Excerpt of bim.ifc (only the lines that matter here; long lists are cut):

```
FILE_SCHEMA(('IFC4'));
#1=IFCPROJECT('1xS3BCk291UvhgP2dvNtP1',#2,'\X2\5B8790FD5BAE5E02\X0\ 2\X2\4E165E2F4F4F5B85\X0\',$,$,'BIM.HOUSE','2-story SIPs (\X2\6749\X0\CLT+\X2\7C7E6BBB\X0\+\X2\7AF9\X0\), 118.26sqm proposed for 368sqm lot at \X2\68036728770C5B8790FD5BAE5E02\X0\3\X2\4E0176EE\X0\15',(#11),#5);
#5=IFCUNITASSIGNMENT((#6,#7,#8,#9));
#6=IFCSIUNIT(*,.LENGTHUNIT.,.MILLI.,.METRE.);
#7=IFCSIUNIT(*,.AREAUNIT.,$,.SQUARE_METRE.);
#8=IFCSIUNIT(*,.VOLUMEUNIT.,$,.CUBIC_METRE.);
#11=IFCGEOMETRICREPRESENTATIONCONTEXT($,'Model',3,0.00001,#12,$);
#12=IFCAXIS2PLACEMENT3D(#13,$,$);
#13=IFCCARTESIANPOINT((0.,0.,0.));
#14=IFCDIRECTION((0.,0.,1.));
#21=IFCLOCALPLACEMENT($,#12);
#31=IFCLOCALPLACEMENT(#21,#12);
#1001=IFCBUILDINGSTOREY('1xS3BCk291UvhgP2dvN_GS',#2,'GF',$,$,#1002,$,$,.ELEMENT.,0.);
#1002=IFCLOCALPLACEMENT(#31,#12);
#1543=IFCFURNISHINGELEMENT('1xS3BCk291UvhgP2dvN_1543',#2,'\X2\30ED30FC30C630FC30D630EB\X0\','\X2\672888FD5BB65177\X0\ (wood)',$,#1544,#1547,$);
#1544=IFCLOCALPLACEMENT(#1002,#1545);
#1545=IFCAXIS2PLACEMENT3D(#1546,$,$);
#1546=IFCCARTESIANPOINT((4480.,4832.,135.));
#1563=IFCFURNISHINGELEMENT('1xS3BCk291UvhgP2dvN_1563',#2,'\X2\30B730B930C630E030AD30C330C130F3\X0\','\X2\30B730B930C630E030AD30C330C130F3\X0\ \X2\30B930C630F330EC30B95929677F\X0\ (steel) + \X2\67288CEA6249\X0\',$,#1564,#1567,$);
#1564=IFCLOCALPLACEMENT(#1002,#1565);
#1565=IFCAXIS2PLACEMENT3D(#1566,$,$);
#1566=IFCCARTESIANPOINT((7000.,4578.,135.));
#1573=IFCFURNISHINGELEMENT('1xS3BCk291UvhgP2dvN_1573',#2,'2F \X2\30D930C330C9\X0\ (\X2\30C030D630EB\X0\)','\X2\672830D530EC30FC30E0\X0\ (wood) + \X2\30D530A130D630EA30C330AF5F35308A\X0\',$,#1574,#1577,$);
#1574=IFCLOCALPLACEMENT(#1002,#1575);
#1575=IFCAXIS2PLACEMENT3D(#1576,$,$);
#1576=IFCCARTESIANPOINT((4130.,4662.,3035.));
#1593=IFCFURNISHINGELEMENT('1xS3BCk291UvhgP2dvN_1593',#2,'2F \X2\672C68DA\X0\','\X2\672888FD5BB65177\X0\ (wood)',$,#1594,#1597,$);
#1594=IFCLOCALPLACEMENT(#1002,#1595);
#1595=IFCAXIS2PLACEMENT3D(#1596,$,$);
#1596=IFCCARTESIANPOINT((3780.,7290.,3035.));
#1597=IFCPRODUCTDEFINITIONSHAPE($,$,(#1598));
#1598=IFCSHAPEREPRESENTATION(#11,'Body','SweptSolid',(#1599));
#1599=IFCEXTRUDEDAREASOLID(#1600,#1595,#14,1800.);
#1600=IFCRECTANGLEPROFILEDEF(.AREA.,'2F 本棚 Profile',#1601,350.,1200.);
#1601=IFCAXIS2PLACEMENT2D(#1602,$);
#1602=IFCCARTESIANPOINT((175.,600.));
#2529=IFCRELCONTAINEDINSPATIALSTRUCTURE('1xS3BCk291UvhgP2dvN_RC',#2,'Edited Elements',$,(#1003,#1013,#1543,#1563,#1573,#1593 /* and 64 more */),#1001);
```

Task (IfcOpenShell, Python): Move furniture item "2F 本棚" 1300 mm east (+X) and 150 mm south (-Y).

```python
import ifcopenshell
import ifcopenshell.api.geometry
import ifcopenshell.util.placement
import ifcopenshell.util.unit

model = ifcopenshell.open("bim.ifc")
unit_scale = ifcopenshell.util.unit.calculate_unit_scale(model)

item = model.by_guid("1xS3BCk291UvhgP2dvN_1593")
matrix = ifcopenshell.util.placement.get_local_placement(item.ObjectPlacement)
matrix[0, 3] += 1.3 / unit_scale
matrix[1, 3] -= 0.15 / unit_scale
ifcopenshell.api.geometry.edit_object_placement(model, product=item, matrix=matrix, is_si=False)

print(ifcopenshell.util.placement.get_local_placement(item.ObjectPlacement).round(3) + 0.0)

model.write("bim_v2.ifc")
```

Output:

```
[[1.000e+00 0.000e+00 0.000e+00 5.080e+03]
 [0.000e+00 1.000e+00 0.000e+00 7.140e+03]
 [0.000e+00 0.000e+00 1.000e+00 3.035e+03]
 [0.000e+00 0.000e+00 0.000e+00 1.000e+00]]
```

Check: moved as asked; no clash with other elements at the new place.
